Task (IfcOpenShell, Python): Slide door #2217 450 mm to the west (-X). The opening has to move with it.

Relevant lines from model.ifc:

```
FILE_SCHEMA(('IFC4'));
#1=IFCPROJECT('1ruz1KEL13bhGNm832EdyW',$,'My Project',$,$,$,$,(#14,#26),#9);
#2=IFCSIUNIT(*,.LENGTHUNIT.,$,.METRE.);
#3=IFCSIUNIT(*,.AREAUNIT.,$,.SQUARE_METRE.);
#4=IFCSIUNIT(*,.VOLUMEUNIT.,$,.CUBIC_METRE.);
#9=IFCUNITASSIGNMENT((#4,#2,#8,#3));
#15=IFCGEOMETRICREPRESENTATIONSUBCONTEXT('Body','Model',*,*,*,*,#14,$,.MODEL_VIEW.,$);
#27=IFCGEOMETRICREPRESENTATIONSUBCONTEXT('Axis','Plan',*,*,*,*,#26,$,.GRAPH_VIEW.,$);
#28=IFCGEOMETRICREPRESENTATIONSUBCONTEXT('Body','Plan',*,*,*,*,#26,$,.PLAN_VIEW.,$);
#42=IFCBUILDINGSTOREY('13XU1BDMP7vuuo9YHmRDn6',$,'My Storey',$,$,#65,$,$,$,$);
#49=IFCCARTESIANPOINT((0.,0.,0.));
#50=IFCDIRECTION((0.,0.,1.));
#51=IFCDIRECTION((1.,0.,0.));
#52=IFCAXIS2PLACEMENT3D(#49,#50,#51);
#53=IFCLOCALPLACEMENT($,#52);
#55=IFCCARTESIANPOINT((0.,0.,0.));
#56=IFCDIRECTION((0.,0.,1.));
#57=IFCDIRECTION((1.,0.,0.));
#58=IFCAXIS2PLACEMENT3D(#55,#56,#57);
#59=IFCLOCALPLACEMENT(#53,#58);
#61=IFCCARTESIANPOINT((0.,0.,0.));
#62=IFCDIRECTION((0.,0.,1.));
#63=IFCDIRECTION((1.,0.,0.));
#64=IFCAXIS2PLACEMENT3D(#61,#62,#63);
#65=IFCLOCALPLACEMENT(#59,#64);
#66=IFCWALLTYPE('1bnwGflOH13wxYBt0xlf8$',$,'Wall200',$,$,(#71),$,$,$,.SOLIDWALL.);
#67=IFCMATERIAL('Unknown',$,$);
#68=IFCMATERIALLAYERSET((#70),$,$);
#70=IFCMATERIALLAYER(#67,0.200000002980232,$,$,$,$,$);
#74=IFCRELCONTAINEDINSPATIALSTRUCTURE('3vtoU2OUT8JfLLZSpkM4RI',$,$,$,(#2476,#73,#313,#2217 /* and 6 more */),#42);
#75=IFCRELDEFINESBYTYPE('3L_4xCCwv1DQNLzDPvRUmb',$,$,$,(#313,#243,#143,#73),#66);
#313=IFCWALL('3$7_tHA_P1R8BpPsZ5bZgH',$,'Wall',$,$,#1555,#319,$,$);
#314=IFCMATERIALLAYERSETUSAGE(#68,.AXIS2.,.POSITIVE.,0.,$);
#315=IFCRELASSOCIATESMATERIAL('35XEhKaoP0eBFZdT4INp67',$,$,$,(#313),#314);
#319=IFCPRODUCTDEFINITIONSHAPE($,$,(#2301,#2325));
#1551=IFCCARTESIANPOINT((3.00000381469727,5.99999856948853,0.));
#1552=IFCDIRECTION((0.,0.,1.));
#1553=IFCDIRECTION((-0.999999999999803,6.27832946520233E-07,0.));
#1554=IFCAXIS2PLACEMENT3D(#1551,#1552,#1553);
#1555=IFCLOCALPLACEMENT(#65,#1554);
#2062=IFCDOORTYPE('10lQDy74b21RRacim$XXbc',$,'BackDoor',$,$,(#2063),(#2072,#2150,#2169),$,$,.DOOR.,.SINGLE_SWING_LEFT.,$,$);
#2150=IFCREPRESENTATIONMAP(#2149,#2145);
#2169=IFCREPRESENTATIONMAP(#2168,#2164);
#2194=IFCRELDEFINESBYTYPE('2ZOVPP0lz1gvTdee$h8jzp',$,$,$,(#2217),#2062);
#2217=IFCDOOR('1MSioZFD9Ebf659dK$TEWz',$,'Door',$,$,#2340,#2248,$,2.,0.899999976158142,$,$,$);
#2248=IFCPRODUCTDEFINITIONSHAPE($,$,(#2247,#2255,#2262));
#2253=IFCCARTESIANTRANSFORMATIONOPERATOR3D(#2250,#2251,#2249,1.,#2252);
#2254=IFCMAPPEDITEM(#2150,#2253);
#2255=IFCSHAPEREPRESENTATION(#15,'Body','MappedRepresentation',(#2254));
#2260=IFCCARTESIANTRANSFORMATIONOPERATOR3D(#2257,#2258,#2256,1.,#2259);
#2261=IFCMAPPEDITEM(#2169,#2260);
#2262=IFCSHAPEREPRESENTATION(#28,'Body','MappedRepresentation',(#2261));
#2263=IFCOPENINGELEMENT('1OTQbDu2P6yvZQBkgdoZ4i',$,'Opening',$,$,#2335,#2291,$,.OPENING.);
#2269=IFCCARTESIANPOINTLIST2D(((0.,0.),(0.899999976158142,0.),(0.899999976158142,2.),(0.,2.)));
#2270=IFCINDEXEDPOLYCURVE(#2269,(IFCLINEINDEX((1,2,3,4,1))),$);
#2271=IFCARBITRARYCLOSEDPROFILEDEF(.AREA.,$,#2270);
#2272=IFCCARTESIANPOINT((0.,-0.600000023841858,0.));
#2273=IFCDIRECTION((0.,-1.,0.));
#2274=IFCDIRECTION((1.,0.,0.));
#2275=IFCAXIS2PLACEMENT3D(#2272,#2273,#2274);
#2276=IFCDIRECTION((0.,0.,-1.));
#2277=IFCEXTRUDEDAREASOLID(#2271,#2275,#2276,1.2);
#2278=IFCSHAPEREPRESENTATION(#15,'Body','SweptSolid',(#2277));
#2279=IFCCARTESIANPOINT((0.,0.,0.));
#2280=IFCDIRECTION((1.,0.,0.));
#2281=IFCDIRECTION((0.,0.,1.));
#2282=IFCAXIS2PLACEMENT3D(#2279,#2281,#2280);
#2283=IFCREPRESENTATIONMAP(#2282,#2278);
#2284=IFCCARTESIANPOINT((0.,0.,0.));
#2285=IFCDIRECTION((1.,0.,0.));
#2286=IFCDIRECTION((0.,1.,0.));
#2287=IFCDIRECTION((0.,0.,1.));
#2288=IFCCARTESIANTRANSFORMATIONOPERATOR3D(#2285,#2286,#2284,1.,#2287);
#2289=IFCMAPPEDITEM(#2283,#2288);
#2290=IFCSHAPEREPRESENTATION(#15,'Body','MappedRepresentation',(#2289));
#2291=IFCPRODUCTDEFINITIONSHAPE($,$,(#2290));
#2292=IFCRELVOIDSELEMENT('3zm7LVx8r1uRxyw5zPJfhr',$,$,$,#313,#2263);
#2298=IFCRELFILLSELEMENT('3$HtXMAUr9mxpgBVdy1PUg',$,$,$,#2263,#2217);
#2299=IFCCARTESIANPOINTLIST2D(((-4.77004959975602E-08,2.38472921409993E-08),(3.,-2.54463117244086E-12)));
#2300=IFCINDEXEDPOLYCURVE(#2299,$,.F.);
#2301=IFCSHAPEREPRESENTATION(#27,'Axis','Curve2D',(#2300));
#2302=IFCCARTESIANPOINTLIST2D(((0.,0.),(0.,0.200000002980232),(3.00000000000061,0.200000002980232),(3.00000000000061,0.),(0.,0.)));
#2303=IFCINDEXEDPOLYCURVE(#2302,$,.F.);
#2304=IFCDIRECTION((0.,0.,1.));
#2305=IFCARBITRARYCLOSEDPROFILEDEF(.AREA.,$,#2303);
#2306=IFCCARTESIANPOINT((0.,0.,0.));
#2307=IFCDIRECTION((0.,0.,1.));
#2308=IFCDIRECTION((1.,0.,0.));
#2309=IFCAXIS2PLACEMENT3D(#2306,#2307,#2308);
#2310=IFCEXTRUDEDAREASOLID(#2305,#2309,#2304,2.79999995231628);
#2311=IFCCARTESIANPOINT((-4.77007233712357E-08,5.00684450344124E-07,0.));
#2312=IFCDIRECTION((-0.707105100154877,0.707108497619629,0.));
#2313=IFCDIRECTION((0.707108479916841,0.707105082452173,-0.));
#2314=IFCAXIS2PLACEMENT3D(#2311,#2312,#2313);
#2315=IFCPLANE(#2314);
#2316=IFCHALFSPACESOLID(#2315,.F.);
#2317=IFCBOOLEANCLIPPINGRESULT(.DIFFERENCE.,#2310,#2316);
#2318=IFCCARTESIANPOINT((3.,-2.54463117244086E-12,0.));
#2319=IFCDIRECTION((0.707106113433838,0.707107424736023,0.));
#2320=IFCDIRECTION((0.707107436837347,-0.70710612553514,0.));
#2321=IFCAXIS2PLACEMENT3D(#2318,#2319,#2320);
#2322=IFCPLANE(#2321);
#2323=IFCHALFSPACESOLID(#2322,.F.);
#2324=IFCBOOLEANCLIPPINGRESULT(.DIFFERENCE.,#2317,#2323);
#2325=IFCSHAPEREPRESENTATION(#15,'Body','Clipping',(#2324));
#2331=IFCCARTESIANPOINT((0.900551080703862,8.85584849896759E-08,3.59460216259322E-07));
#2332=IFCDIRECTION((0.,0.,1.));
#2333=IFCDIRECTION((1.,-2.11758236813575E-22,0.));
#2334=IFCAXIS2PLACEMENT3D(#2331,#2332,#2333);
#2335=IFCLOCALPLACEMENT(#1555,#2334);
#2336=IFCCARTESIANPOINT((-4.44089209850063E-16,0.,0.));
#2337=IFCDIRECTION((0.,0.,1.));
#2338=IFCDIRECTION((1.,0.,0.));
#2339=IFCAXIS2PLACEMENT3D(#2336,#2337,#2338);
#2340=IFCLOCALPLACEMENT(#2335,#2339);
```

```python
import ifcopenshell
import ifcopenshell.api.geometry
import ifcopenshell.util.placement

model = ifcopenshell.open("model.ifc")

door = model.by_id(2217)
opening = door.FillsVoids[0].RelatingOpeningElement
wall = opening.VoidsElements[0].RelatingBuildingElement

wall_matrix = ifcopenshell.util.placement.get_local_placement(wall.ObjectPlacement)
shift = wall_matrix[:3, 0] * 0.45
before = ifcopenshell.util.placement.get_local_placement(door.ObjectPlacement)[:3, 3].copy()

# The door is placed relative to its opening, so it follows when the opening moves.
matrix = ifcopenshell.util.placement.get_local_placement(opening.ObjectPlacement)
matrix[:3, 3] += shift
ifcopenshell.api.geometry.edit_object_placement(
    model, product=opening, matrix=matrix, is_si=False, should_transform_children=True
)

after = ifcopenshell.util.placement.get_local_placement(door.ObjectPlacement)[:3, 3]
print("door moved by", (after - before).round(3) + 0.0)

model.write("model-out.ifc")
```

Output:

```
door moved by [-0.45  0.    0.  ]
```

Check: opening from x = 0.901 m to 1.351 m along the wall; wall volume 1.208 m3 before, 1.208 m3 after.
